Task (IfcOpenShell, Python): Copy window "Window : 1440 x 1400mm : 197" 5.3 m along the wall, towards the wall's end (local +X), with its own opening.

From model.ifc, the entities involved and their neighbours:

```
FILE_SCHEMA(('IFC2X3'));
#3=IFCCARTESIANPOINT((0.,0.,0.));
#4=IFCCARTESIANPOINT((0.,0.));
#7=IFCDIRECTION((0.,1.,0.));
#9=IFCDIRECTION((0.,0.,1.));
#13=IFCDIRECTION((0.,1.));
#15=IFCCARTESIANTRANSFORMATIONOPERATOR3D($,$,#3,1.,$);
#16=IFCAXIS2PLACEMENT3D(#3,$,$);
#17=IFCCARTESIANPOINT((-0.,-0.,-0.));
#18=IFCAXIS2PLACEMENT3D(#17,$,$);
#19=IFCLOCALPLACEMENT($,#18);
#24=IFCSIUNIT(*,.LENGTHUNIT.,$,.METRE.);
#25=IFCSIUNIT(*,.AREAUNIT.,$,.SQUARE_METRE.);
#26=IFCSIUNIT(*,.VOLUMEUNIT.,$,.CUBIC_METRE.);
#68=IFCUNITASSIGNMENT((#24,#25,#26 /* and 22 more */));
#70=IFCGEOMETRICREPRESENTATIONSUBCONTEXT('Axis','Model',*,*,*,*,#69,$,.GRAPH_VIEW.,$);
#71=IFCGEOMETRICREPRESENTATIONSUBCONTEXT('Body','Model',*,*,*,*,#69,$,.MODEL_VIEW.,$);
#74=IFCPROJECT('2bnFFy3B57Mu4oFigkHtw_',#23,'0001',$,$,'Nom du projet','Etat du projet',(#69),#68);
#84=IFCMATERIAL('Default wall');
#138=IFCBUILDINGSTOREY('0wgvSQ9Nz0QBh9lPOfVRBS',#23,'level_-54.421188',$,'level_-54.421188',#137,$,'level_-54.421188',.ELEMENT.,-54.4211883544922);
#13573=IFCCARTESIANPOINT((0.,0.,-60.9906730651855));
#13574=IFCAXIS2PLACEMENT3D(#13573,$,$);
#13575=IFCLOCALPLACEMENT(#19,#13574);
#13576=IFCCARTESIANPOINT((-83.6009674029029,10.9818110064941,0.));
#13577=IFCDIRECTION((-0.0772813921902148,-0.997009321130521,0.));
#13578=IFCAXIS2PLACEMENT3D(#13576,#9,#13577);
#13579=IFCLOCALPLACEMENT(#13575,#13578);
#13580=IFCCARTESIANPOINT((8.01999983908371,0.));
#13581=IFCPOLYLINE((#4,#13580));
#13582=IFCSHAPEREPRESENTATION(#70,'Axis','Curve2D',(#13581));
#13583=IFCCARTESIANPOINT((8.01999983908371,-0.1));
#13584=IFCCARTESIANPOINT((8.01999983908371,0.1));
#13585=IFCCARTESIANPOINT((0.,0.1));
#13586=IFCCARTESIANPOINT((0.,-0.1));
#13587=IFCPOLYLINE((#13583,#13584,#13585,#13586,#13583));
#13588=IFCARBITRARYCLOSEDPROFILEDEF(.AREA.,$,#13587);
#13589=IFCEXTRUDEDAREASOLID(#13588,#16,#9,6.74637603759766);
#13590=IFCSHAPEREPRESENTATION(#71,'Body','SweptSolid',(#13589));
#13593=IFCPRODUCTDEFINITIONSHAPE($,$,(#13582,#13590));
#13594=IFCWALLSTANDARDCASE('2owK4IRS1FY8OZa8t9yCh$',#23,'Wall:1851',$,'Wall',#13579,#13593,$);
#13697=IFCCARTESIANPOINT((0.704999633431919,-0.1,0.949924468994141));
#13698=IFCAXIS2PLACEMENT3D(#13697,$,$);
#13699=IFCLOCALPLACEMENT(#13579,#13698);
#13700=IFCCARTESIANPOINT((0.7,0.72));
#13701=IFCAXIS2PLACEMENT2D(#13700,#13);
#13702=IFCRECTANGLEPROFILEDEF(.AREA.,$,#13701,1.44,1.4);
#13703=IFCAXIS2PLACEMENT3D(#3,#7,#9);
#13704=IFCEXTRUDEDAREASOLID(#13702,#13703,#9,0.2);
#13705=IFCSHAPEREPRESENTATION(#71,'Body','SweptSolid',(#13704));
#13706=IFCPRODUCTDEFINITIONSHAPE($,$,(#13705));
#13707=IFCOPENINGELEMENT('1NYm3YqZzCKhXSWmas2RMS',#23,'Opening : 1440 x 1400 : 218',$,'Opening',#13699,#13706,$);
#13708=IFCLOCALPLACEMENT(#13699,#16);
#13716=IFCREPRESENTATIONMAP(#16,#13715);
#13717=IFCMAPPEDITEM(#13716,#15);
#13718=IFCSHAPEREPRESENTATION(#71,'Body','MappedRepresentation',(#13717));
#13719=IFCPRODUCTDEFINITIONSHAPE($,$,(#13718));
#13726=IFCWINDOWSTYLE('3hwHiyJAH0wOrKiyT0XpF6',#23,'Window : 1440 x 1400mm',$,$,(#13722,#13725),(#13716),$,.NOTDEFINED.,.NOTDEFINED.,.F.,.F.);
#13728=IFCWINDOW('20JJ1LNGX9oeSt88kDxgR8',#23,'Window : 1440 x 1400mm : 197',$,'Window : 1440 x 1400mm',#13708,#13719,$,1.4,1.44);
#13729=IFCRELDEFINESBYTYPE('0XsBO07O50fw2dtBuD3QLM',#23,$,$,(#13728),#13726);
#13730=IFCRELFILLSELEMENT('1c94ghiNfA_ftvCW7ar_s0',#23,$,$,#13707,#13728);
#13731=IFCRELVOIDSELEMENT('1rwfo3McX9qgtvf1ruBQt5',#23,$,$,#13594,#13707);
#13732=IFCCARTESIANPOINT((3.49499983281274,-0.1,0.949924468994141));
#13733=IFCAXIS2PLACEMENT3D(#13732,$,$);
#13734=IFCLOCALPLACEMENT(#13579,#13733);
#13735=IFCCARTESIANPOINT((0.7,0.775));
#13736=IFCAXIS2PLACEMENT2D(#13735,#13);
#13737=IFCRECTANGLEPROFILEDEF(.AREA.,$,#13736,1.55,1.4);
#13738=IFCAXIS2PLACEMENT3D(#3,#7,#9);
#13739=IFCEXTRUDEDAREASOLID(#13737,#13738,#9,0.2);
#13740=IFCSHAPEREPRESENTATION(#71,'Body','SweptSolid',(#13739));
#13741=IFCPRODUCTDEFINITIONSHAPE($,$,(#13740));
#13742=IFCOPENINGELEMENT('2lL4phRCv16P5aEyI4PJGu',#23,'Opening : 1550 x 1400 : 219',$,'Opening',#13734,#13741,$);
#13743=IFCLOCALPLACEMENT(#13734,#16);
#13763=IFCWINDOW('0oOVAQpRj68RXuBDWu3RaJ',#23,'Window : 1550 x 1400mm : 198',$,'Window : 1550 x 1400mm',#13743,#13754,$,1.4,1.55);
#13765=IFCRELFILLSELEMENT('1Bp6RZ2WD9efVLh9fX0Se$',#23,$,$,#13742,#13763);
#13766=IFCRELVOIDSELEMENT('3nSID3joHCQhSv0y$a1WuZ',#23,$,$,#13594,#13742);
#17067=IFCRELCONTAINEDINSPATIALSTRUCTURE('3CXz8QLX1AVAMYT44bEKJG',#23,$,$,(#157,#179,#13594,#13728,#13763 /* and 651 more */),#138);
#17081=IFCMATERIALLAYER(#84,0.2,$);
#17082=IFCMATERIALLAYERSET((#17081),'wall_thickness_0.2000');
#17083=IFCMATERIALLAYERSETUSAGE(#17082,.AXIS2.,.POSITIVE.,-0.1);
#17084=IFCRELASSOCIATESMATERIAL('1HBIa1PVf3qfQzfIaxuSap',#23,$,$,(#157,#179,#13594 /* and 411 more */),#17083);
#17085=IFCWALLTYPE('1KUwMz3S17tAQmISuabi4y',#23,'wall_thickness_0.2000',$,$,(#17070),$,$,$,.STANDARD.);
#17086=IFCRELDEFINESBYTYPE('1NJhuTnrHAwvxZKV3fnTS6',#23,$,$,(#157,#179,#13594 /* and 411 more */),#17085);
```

```python
import ifcopenshell
import ifcopenshell.api.feature
import ifcopenshell.api.geometry
import ifcopenshell.api.root
import ifcopenshell.geom
import ifcopenshell.util.element
import ifcopenshell.util.placement
import ifcopenshell.util.shape
import ifcopenshell.util.unit

model = ifcopenshell.open("model.ifc")
unit_scale = ifcopenshell.util.unit.calculate_unit_scale(model)
settings = ifcopenshell.geom.settings()


def volume(element):
    """Net volume in cubic metres, openings subtracted."""
    shape = ifcopenshell.geom.create_shape(settings, element)
    return ifcopenshell.util.shape.get_volume(shape.geometry)


window = model.by_id(13728)
opening = window.FillsVoids[0].RelatingOpeningElement
wall = opening.VoidsElements[0].RelatingBuildingElement
before = volume(wall)
shift = ifcopenshell.util.placement.get_local_placement(wall.ObjectPlacement)[:3, 0] * 5.3 / unit_scale

# copy_class copies the void relationship, type, container and properties, but no geometry.
new_opening = ifcopenshell.api.root.copy_class(model, product=opening)
new_opening.Representation = ifcopenshell.util.element.copy_deep(
    model, opening.Representation, exclude=["IfcGeometricRepresentationContext", "IfcRepresentationMap"]
)
new_opening.Name = "Opening : 1440 x 1400"
new_window = ifcopenshell.api.root.copy_class(model, product=window)
new_window.Representation = ifcopenshell.util.element.copy_deep(
    model, window.Representation, exclude=["IfcGeometricRepresentationContext", "IfcRepresentationMap"]
)
new_window.Name = "Window : 1440 x 1400mm"
fills = ifcopenshell.api.feature.add_filling(model, opening=new_opening, element=new_window)
fills.OwnerHistory = new_window.OwnerHistory  # required in IFC2X3

for old, new in ((opening, new_opening), (window, new_window)):
    matrix = ifcopenshell.util.placement.get_local_placement(old.ObjectPlacement)
    matrix[:3, 3] += shift
    ifcopenshell.api.geometry.edit_object_placement(model, product=new, matrix=matrix, is_si=False)

after = volume(wall)

print(f"wall volume {before:.3f} -> {after:.3f} m3")

model.write("model_updated.ifc")
```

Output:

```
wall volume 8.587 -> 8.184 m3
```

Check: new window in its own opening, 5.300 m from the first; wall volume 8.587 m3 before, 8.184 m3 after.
